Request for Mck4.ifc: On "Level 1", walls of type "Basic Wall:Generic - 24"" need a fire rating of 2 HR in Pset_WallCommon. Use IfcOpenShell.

First a look at what the model holds.

```python
import ifcopenshell
import ifcopenshell.util.element

model = ifcopenshell.open("Mck4.ifc")
print(model.schema)
storey = next(s for s in model.by_type("IfcBuildingStorey") if s.Name == "Level 1")
walls = [e for e in ifcopenshell.util.element.get_decomposition(storey) if e.is_a("IfcWall")]
seen = {}
for e in walls:
    element_type = ifcopenshell.util.element.get_type(e)
    key = (element_type.Name if element_type != e and element_type else None, ifcopenshell.util.element.get_pset(e, "Pset_WallCommon", "FireRating"))
    seen[key] = seen.get(key, 0) + 1
for (name, value), count in sorted(seen.items(), key=str):
    print(count, "x", name, "|", value)
```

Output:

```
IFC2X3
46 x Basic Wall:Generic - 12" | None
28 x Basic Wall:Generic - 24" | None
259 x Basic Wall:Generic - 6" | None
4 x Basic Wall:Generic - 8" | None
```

```python
import ifcopenshell
import ifcopenshell.api.pset
import ifcopenshell.util.element

model = ifcopenshell.open("Mck4.ifc")

storey = next(s for s in model.by_type("IfcBuildingStorey") if s.Name == "Level 1")
walls = [e for e in ifcopenshell.util.element.get_decomposition(storey) if e.is_a("IfcWall")]

count = 0
for e in walls:
    element_type = ifcopenshell.util.element.get_type(e)
    if element_type in (None, e) or element_type.Name != 'Basic Wall:Generic - 24"':
        continue
    # add_pset returns the element's existing set when there is one.
    pset = ifcopenshell.api.pset.add_pset(model, product=e, name="Pset_WallCommon")
    ifcopenshell.api.pset.edit_pset(model, pset=pset, properties={"FireRating": "2 HR"})
    count += 1

print(count, "walls updated")

model.write("Mck4_rev.ifc")
```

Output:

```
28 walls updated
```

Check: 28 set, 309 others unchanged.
